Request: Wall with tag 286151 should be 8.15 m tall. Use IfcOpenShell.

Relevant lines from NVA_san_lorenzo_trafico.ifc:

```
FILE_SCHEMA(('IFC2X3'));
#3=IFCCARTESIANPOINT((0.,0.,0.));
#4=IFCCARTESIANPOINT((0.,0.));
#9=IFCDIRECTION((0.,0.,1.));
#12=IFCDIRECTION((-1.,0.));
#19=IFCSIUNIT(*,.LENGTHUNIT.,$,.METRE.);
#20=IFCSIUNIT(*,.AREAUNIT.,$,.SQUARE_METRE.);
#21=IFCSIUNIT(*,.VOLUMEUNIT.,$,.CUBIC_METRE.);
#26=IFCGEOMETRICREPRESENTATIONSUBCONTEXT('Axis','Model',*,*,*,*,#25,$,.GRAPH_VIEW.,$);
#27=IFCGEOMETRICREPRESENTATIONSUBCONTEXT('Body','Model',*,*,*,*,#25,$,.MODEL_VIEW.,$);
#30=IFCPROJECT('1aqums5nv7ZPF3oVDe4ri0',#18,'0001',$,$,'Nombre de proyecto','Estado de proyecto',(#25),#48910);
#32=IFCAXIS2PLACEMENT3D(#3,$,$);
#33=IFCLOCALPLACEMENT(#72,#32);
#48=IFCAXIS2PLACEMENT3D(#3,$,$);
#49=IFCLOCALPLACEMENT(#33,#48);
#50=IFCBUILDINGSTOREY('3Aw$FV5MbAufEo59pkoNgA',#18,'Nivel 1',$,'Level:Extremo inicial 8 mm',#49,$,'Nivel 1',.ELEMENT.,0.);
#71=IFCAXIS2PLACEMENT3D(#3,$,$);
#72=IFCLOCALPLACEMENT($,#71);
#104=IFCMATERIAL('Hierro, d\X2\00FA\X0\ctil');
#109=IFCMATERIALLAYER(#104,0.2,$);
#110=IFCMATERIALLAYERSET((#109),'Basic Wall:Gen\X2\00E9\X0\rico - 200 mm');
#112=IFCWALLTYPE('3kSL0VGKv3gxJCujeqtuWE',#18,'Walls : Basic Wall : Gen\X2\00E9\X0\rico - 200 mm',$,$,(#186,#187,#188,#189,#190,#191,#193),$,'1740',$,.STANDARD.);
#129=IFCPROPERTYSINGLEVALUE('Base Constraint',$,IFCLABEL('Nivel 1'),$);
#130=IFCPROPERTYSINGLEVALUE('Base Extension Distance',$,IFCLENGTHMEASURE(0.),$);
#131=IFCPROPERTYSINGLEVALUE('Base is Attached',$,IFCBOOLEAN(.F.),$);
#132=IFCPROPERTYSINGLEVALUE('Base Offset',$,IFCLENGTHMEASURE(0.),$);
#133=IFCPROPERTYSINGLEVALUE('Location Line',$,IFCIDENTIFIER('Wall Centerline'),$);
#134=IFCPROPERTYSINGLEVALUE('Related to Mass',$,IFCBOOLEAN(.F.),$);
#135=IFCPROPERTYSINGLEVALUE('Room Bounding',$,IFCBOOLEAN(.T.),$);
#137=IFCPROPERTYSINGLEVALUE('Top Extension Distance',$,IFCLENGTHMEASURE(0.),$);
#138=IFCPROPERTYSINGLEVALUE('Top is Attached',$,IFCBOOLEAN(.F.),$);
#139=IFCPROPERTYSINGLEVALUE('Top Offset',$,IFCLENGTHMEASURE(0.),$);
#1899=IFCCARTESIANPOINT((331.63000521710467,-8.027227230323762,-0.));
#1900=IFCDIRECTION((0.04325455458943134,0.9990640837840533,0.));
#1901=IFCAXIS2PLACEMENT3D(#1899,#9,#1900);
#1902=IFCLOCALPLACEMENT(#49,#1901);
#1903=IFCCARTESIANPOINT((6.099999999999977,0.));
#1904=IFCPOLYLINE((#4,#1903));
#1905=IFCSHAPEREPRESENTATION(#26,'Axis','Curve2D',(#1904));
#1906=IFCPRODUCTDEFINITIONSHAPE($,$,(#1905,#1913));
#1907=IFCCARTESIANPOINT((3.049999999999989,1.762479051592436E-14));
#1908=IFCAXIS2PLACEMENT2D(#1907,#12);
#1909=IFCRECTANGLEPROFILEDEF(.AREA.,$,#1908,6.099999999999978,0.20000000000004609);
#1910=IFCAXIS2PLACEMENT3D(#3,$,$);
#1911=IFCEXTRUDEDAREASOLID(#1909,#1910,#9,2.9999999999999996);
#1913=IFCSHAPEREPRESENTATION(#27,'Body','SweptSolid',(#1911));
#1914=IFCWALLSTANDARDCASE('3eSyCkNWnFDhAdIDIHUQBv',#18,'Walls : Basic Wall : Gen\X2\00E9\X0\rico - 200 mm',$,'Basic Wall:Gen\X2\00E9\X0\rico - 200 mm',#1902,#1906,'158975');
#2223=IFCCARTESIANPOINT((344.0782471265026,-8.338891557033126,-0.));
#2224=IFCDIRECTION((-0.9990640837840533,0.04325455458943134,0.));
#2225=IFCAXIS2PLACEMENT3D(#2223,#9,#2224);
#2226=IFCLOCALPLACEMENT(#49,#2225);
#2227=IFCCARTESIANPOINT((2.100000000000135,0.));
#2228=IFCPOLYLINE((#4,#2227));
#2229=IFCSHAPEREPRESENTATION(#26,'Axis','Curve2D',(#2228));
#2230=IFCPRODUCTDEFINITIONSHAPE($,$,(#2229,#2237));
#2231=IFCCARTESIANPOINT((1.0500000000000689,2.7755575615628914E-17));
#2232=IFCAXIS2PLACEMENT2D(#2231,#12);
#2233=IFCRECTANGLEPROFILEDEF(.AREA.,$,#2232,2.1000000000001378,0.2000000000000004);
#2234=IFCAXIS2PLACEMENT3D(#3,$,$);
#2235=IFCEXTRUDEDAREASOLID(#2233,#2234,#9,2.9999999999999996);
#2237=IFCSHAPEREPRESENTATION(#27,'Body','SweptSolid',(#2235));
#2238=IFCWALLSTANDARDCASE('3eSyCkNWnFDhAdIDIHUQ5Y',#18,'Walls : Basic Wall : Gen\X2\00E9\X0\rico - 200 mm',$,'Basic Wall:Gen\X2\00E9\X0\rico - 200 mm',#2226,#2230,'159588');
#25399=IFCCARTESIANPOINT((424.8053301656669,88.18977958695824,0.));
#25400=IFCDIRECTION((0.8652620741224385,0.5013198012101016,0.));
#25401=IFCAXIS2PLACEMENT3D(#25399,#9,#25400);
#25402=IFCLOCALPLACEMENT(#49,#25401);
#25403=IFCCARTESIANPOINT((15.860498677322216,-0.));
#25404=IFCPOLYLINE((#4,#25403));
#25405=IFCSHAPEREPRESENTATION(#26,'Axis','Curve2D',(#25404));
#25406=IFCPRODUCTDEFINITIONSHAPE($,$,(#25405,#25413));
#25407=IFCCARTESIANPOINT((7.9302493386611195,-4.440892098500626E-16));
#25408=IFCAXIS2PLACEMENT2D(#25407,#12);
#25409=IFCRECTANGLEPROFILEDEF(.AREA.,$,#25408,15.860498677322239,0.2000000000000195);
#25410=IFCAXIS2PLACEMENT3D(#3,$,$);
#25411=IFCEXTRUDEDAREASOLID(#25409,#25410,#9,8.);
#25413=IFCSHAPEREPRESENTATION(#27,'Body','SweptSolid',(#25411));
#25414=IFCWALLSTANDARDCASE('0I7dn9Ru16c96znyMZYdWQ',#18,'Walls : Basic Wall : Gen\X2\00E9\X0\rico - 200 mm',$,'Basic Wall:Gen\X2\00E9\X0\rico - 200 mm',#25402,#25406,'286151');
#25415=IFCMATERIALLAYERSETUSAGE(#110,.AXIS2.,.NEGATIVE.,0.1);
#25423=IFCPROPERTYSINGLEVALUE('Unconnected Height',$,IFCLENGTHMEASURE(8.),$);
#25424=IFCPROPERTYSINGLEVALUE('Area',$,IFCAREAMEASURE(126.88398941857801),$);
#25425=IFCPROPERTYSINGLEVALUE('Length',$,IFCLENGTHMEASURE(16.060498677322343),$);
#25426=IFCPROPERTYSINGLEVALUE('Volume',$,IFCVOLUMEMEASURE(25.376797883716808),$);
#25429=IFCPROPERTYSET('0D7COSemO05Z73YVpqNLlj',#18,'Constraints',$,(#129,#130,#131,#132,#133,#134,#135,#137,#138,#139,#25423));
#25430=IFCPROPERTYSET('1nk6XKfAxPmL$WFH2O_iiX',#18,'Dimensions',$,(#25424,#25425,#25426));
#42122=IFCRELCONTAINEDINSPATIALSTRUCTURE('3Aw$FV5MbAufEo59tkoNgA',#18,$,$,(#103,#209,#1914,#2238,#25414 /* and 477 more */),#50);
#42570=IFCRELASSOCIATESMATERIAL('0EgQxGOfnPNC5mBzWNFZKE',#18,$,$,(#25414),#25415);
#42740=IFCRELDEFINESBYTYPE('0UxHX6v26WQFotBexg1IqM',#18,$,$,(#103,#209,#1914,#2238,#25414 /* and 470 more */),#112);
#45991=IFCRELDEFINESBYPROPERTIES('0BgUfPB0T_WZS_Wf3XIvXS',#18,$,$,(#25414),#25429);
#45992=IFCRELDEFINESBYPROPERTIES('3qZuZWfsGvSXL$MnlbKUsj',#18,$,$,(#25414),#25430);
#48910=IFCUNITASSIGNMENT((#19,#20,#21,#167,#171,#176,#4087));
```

```python
import ifcopenshell
import ifcopenshell.api.pset
import ifcopenshell.geom
import ifcopenshell.util.element
import ifcopenshell.util.representation
import ifcopenshell.util.shape
import ifcopenshell.util.unit

model = ifcopenshell.open("NVA_san_lorenzo_trafico.ifc")
area_scale = ifcopenshell.util.unit.calculate_unit_scale(model, "AREAUNIT")
volume_scale = ifcopenshell.util.unit.calculate_unit_scale(model, "VOLUMEUNIT")
settings = ifcopenshell.geom.settings()


def volume(element):
    """Net volume in cubic metres, openings subtracted."""
    shape = ifcopenshell.geom.create_shape(settings, element)
    return ifcopenshell.util.shape.get_volume(shape.geometry)


wall = model.by_guid("0I7dn9Ru16c96znyMZYdWQ")
before = volume(wall)

body = ifcopenshell.util.representation.get_representation(wall, "Model", "Body")
solid = body.Items[0]
old_height = solid.Depth
solid.Depth = 8.15
after = volume(wall)
thickness = 0.2  # wall thickness in metres

# Update the stored height, areas and volumes.
pset = model.by_id(ifcopenshell.util.element.get_pset(wall, "Constraints", should_inherit=False)["id"])
ifcopenshell.api.pset.edit_pset(model, pset=pset, properties={
    "Unconnected Height": model.create_entity("IfcLengthMeasure", solid.Depth),
})
pset = model.by_id(ifcopenshell.util.element.get_pset(wall, "Dimensions", should_inherit=False)["id"])
ifcopenshell.api.pset.edit_pset(model, pset=pset, properties={
    "Area": model.create_entity("IfcAreaMeasure", after / thickness / area_scale),
    "Volume": model.create_entity("IfcVolumeMeasure", after / volume_scale),
})

print(f"height {old_height:g} -> {solid.Depth:g}, volume {before:.3f} -> {after:.3f} m3")

model.write("NVA_san_lorenzo_trafico_v2.ifc")
```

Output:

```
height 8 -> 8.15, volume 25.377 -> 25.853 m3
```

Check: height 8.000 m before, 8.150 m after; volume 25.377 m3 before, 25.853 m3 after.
